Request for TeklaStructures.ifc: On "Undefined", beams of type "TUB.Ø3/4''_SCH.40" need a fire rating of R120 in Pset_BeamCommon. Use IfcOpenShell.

First a look at what the model holds.

```python
import ifcopenshell
import ifcopenshell.util.element

model = ifcopenshell.open("TeklaStructures.ifc")
print(model.schema)
storey = next(s for s in model.by_type("IfcBuildingStorey") if s.Name == "Undefined")
beams = [e for e in ifcopenshell.util.element.get_decomposition(storey) if e.is_a("IfcBeam")]
seen = {}
for e in beams:
    element_type = ifcopenshell.util.element.get_type(e)
    key = (element_type.Name if element_type != e and element_type else None, ifcopenshell.util.element.get_pset(e, "Pset_BeamCommon", "FireRating"))
    seen[key] = seen.get(key, 0) + 1
for (name, value), count in sorted(seen.items(), key=str):
    print(count, "x", name, "|", value)
```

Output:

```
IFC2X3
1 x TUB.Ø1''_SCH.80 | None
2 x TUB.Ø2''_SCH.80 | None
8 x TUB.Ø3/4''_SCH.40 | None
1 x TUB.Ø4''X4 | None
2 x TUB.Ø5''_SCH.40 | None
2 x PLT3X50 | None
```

```python
import ifcopenshell
import ifcopenshell.api.pset
import ifcopenshell.util.element

model = ifcopenshell.open("TeklaStructures.ifc")

storey = next(s for s in model.by_type("IfcBuildingStorey") if s.Name == "Undefined")
beams = [e for e in ifcopenshell.util.element.get_decomposition(storey) if e.is_a("IfcBeam")]

count = 0
for e in beams:
    element_type = ifcopenshell.util.element.get_type(e)
    if element_type in (None, e) or element_type.Name != "TUB.Ø3/4''_SCH.40":
        continue
    # add_pset returns the element's existing set when there is one.
    pset = ifcopenshell.api.pset.add_pset(model, product=e, name="Pset_BeamCommon")
    ifcopenshell.api.pset.edit_pset(model, pset=pset, properties={"FireRating": "R120"})
    count += 1

print(count, "beams updated")

model.write("TeklaStructures-out.ifc")
```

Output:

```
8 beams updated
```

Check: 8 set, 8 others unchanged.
